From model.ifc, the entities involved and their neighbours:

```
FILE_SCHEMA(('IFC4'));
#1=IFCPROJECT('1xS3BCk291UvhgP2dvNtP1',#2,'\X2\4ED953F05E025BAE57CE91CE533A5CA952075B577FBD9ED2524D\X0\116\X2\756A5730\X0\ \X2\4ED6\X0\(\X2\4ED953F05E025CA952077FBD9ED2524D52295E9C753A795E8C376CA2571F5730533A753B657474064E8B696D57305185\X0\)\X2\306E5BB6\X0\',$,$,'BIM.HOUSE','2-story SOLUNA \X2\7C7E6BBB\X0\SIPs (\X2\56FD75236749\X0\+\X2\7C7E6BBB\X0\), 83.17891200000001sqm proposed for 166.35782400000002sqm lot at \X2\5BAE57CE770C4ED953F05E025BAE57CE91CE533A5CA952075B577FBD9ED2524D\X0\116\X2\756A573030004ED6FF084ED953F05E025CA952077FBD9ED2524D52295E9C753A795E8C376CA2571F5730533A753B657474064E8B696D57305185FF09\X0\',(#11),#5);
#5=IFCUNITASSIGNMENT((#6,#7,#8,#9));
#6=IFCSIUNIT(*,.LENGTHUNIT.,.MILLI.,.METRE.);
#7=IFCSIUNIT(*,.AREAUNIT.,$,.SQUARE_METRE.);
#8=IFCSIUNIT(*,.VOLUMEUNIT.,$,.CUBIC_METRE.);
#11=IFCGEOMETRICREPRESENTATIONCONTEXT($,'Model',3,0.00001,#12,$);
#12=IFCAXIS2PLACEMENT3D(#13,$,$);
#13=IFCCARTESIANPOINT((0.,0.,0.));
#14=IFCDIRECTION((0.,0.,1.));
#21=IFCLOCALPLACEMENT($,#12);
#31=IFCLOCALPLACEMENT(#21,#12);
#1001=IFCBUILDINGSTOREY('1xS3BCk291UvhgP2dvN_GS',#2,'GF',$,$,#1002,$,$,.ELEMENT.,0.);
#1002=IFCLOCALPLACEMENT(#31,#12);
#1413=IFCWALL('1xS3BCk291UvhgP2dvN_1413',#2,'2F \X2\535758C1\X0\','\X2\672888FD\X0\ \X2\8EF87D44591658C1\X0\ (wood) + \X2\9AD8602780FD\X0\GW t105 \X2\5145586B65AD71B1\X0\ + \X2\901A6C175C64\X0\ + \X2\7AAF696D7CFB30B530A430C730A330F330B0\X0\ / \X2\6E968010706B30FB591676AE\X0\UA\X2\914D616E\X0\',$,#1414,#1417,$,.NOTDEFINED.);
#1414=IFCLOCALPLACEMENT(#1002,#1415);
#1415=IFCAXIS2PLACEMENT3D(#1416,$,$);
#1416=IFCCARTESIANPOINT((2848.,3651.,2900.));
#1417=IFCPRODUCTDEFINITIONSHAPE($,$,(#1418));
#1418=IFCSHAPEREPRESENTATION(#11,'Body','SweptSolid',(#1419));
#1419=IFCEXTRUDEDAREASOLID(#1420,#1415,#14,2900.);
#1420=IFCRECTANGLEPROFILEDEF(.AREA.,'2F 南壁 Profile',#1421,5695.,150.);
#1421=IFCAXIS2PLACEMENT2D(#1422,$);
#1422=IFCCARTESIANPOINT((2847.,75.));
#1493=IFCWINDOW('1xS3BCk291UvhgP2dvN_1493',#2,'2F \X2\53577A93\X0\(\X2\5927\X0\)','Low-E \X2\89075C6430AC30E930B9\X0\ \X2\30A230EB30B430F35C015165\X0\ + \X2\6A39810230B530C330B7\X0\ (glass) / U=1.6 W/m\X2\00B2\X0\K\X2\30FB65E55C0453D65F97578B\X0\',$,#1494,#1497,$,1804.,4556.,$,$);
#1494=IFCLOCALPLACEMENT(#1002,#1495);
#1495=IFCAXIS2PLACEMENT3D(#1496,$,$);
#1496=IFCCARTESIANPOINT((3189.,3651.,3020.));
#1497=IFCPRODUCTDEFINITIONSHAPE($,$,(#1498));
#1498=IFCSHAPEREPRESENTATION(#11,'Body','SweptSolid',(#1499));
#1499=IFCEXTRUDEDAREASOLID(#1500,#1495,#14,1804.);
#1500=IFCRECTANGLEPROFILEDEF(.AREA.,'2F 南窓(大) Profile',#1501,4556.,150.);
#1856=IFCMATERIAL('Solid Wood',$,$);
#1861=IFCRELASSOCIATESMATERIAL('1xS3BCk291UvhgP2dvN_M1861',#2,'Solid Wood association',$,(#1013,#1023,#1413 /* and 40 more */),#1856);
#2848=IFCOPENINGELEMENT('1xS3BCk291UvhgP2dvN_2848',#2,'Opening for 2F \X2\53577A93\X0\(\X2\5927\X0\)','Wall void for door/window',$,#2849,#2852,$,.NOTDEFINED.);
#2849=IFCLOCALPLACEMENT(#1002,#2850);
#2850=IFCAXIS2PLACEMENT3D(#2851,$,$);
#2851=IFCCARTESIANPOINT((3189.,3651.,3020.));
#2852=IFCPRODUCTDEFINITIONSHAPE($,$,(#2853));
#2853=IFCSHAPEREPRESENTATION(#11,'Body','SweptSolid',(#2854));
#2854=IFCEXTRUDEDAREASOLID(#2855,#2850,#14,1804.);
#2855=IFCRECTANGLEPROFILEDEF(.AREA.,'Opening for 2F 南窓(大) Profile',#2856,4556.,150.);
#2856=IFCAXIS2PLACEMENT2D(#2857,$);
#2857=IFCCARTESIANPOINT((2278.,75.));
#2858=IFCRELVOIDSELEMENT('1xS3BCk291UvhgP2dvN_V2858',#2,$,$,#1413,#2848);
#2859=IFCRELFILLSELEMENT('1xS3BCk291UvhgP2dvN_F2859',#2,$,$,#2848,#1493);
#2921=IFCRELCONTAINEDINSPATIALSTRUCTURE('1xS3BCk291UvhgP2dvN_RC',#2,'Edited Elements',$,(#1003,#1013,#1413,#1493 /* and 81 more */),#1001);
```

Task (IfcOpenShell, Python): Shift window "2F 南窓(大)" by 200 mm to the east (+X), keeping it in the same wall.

```python
import ifcopenshell
import ifcopenshell.api.geometry
import ifcopenshell.util.placement

model = ifcopenshell.open("model.ifc")

window = model.by_guid("1xS3BCk291UvhgP2dvN_1493")
opening = window.FillsVoids[0].RelatingOpeningElement
wall = opening.VoidsElements[0].RelatingBuildingElement

wall_matrix = ifcopenshell.util.placement.get_local_placement(wall.ObjectPlacement)
shift = wall_matrix[:3, 0] * 200.0
before = ifcopenshell.util.placement.get_local_placement(window.ObjectPlacement)[:3, 3].copy()

# The window is not placed relative to its opening, so move both.
for product in (opening, window):
    matrix = ifcopenshell.util.placement.get_local_placement(product.ObjectPlacement)
    matrix[:3, 3] += shift
    ifcopenshell.api.geometry.edit_object_placement(model, product=product, matrix=matrix, is_si=False)

after = ifcopenshell.util.placement.get_local_placement(window.ObjectPlacement)[:3, 3]
print("window moved by", (after - before).round(3) + 0.0)

model.write("model_v2.ifc")
```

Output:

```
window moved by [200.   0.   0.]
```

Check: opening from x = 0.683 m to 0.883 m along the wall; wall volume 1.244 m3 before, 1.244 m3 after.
